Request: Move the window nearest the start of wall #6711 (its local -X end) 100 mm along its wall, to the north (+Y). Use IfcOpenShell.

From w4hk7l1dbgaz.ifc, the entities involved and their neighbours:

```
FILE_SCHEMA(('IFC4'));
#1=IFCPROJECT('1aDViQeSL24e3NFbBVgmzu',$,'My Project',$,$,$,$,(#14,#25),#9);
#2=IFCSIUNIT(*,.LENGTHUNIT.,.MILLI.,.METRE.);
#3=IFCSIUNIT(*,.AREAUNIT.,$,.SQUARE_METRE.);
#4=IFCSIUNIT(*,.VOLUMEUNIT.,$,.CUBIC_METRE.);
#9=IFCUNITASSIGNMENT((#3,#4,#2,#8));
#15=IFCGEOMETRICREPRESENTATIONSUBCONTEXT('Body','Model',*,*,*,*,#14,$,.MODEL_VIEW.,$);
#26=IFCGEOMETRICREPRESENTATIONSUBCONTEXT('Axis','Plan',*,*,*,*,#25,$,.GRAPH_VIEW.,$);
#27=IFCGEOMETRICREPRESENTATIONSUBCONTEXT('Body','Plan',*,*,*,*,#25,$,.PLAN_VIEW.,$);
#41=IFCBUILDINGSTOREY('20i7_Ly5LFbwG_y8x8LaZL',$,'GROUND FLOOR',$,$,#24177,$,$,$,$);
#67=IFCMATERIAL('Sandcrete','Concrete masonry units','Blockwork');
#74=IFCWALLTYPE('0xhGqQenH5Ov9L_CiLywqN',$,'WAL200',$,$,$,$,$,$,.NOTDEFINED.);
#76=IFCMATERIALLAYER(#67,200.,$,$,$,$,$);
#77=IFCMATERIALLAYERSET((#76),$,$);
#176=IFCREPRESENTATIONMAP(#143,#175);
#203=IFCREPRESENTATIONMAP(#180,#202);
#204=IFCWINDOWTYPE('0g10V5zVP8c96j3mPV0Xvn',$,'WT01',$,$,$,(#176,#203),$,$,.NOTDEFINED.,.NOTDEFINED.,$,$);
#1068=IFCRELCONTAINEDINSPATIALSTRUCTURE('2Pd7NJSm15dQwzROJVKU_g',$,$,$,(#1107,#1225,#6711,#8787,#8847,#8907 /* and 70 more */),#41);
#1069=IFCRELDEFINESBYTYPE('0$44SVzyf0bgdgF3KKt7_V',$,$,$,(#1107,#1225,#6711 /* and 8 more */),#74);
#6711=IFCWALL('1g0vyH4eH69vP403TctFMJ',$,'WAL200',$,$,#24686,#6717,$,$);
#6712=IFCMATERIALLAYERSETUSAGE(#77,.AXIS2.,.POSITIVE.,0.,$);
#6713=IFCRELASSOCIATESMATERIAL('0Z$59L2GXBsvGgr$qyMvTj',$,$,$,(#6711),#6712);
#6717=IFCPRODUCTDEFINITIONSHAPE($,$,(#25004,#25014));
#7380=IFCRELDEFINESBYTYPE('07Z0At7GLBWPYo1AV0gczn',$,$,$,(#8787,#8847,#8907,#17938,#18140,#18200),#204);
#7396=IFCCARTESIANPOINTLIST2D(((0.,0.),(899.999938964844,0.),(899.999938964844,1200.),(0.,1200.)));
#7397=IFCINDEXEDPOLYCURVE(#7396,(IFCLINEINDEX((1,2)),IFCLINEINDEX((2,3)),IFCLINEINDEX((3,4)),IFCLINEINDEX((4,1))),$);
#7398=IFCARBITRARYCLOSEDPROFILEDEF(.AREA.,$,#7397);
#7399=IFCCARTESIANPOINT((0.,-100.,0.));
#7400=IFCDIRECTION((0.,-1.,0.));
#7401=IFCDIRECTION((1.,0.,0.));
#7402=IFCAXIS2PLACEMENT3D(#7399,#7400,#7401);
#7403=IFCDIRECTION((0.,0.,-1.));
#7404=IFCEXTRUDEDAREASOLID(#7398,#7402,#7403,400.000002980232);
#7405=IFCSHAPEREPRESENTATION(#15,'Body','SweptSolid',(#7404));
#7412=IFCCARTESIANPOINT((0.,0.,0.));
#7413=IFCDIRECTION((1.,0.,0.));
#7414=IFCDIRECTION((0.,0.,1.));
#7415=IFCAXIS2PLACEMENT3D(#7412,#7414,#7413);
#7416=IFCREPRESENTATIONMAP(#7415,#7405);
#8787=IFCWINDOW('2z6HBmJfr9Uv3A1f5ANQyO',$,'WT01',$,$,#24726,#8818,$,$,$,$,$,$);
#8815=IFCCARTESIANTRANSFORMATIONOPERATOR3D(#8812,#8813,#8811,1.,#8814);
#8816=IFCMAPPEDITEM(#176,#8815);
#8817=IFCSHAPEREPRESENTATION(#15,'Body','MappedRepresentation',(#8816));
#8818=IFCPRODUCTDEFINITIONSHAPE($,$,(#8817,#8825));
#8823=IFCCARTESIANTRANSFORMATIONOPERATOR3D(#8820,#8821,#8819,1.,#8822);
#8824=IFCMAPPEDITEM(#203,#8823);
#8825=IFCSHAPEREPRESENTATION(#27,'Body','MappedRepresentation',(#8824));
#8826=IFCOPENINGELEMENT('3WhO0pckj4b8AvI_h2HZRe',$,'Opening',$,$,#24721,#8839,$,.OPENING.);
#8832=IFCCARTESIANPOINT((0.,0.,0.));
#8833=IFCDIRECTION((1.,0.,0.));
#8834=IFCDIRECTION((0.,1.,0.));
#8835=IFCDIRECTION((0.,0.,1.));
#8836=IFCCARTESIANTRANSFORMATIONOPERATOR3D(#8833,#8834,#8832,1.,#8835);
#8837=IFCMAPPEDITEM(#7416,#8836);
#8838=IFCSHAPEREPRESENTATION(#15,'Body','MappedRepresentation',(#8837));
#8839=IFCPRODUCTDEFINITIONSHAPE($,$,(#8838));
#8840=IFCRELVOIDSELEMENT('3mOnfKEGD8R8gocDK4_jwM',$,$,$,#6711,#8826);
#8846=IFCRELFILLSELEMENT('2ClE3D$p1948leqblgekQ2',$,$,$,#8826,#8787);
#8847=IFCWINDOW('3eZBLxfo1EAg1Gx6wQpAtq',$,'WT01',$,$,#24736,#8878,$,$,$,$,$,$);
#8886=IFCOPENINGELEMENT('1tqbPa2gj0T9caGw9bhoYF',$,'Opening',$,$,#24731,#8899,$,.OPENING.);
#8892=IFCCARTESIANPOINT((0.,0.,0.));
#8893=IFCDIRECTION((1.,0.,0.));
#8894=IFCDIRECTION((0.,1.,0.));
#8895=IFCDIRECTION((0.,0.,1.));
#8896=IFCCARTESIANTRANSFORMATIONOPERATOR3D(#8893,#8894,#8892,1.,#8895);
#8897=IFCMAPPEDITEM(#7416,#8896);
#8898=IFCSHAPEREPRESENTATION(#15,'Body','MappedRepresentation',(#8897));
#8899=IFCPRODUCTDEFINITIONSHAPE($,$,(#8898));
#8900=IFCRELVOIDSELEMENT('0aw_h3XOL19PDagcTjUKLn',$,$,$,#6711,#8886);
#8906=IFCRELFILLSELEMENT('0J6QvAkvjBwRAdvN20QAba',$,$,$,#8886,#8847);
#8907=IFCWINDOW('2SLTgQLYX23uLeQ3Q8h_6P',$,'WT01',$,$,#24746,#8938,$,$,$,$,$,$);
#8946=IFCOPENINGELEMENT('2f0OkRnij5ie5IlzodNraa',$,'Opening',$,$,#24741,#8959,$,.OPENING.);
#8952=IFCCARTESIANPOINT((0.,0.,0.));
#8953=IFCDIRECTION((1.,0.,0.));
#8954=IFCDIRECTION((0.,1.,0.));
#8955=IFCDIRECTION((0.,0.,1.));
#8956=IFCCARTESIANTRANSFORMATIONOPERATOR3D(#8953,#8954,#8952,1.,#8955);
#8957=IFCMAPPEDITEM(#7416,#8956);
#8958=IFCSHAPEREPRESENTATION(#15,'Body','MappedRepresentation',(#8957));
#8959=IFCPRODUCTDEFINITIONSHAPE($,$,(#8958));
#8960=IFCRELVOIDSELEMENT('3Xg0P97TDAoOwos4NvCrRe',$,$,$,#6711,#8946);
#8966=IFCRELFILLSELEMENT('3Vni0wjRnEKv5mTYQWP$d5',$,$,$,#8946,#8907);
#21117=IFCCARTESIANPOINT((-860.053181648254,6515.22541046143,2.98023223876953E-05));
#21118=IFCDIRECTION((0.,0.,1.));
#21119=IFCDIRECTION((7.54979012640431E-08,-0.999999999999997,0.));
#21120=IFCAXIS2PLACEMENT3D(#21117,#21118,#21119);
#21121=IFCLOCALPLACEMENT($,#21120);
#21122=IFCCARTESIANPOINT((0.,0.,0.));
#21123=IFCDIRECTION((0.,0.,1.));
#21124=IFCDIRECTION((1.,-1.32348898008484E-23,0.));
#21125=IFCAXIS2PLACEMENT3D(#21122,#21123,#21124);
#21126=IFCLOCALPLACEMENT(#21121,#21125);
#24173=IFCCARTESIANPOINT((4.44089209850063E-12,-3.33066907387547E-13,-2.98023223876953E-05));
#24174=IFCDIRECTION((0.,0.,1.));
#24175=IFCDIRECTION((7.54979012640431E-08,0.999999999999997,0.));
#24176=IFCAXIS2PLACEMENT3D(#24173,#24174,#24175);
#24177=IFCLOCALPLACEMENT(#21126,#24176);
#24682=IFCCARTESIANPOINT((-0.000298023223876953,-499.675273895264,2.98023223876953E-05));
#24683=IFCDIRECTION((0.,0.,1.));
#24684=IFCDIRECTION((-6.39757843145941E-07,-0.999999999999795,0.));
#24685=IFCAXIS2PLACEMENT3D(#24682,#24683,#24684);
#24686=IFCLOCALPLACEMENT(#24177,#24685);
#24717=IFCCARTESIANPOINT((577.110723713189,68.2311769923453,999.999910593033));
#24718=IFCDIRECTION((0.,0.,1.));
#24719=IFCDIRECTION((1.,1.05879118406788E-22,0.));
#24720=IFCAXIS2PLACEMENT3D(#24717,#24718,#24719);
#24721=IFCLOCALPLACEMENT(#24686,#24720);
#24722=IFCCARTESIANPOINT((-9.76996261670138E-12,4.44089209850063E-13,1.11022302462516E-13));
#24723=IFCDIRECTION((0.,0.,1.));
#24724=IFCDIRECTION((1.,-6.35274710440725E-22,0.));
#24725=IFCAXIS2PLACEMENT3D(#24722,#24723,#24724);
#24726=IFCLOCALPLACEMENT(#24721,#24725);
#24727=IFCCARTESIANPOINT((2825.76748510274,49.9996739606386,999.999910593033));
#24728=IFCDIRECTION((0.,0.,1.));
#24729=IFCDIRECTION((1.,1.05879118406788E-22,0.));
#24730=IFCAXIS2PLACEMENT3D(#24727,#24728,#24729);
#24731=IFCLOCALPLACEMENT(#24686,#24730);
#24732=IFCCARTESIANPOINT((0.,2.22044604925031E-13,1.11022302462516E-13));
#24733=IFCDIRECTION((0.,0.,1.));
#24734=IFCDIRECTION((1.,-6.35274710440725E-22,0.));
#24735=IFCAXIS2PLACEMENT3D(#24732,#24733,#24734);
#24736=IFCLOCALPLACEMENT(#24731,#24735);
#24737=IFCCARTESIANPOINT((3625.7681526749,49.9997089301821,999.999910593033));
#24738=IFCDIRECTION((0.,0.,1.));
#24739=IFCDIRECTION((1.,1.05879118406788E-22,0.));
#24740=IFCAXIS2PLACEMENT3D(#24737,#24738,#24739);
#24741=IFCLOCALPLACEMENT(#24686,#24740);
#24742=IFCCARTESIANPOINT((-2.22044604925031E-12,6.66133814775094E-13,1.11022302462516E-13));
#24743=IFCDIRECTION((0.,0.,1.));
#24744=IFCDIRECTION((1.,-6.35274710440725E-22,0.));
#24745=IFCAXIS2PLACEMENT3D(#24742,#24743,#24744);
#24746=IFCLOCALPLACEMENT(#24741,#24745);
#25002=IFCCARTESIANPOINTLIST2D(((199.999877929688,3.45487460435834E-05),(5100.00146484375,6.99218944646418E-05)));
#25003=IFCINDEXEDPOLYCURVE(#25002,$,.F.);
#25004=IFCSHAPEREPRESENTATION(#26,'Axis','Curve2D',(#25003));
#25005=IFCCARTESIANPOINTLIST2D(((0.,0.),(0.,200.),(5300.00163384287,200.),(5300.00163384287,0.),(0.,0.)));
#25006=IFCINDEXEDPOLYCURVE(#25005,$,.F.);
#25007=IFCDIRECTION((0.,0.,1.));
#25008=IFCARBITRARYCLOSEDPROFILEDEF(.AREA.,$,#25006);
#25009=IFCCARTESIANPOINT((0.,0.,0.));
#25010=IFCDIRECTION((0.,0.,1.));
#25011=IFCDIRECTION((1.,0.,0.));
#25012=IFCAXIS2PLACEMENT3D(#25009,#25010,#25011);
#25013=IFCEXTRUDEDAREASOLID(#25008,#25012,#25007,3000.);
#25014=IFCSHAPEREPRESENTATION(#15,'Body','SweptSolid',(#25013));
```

```python
import ifcopenshell
import ifcopenshell.api.geometry
import ifcopenshell.util.placement
import ifcopenshell.util.unit

model = ifcopenshell.open("w4hk7l1dbgaz.ifc")
unit_scale = ifcopenshell.util.unit.calculate_unit_scale(model)

window = model.by_guid("2z6HBmJfr9Uv3A1f5ANQyO")
opening = window.FillsVoids[0].RelatingOpeningElement
wall = opening.VoidsElements[0].RelatingBuildingElement

wall_matrix = ifcopenshell.util.placement.get_local_placement(wall.ObjectPlacement)
shift = wall_matrix[:3, 0] * -0.1 / unit_scale
before = ifcopenshell.util.placement.get_local_placement(window.ObjectPlacement)[:3, 3].copy()

# The window is placed relative to its opening, so it follows when the opening moves.
matrix = ifcopenshell.util.placement.get_local_placement(opening.ObjectPlacement)
matrix[:3, 3] += shift
ifcopenshell.api.geometry.edit_object_placement(
    model, product=opening, matrix=matrix, is_si=False, should_transform_children=True
)

after = ifcopenshell.util.placement.get_local_placement(window.ObjectPlacement)[:3, 3]
print("window moved by", (after - before).round(3) + 0.0)

model.write("w4hk7l1dbgaz_updated.ifc")
```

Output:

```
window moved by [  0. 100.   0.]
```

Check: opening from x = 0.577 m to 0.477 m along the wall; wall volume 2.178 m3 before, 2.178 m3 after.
